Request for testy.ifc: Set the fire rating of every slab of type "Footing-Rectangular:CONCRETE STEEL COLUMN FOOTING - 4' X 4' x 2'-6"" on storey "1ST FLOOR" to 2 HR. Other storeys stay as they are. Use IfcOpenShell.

First a look at what the model holds.

```python
import ifcopenshell
import ifcopenshell.util.element

model = ifcopenshell.open("testy.ifc")
print(model.schema)
storey = next(s for s in model.by_type("IfcBuildingStorey") if s.Name == "1ST FLOOR")
slabs = [e for e in ifcopenshell.util.element.get_decomposition(storey) if e.is_a("IfcSlab")]
seen = {}
for e in slabs:
    element_type = ifcopenshell.util.element.get_type(e)
    key = (element_type.Name if element_type != e and element_type else None, ifcopenshell.util.element.get_pset(e, "Pset_SlabCommon", "FireRating"))
    seen[key] = seen.get(key, 0) + 1
for (name, value), count in sorted(seen.items(), key=str):
    print(count, "x", name, "|", value)
```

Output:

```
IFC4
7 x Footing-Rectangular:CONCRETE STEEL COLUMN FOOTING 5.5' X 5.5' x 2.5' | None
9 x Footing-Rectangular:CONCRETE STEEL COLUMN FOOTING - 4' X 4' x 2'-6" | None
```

```python
import ifcopenshell
import ifcopenshell.api.pset
import ifcopenshell.util.element

model = ifcopenshell.open("testy.ifc")

storey = next(s for s in model.by_type("IfcBuildingStorey") if s.Name == "1ST FLOOR")
slabs = [e for e in ifcopenshell.util.element.get_decomposition(storey) if e.is_a("IfcSlab")]

count = 0
for e in slabs:
    element_type = ifcopenshell.util.element.get_type(e)
    if element_type in (None, e) or element_type.Name != 'Footing-Rectangular:CONCRETE STEEL COLUMN FOOTING - 4\' X 4\' x 2\'-6"':
        continue
    # add_pset returns the element's existing set when there is one.
    pset = ifcopenshell.api.pset.add_pset(model, product=e, name="Pset_SlabCommon")
    ifcopenshell.api.pset.edit_pset(model, pset=pset, properties={"FireRating": "2 HR"})
    count += 1

print(count, "slabs updated")

model.write("testy_edited.ifc")
```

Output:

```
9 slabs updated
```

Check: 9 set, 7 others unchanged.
